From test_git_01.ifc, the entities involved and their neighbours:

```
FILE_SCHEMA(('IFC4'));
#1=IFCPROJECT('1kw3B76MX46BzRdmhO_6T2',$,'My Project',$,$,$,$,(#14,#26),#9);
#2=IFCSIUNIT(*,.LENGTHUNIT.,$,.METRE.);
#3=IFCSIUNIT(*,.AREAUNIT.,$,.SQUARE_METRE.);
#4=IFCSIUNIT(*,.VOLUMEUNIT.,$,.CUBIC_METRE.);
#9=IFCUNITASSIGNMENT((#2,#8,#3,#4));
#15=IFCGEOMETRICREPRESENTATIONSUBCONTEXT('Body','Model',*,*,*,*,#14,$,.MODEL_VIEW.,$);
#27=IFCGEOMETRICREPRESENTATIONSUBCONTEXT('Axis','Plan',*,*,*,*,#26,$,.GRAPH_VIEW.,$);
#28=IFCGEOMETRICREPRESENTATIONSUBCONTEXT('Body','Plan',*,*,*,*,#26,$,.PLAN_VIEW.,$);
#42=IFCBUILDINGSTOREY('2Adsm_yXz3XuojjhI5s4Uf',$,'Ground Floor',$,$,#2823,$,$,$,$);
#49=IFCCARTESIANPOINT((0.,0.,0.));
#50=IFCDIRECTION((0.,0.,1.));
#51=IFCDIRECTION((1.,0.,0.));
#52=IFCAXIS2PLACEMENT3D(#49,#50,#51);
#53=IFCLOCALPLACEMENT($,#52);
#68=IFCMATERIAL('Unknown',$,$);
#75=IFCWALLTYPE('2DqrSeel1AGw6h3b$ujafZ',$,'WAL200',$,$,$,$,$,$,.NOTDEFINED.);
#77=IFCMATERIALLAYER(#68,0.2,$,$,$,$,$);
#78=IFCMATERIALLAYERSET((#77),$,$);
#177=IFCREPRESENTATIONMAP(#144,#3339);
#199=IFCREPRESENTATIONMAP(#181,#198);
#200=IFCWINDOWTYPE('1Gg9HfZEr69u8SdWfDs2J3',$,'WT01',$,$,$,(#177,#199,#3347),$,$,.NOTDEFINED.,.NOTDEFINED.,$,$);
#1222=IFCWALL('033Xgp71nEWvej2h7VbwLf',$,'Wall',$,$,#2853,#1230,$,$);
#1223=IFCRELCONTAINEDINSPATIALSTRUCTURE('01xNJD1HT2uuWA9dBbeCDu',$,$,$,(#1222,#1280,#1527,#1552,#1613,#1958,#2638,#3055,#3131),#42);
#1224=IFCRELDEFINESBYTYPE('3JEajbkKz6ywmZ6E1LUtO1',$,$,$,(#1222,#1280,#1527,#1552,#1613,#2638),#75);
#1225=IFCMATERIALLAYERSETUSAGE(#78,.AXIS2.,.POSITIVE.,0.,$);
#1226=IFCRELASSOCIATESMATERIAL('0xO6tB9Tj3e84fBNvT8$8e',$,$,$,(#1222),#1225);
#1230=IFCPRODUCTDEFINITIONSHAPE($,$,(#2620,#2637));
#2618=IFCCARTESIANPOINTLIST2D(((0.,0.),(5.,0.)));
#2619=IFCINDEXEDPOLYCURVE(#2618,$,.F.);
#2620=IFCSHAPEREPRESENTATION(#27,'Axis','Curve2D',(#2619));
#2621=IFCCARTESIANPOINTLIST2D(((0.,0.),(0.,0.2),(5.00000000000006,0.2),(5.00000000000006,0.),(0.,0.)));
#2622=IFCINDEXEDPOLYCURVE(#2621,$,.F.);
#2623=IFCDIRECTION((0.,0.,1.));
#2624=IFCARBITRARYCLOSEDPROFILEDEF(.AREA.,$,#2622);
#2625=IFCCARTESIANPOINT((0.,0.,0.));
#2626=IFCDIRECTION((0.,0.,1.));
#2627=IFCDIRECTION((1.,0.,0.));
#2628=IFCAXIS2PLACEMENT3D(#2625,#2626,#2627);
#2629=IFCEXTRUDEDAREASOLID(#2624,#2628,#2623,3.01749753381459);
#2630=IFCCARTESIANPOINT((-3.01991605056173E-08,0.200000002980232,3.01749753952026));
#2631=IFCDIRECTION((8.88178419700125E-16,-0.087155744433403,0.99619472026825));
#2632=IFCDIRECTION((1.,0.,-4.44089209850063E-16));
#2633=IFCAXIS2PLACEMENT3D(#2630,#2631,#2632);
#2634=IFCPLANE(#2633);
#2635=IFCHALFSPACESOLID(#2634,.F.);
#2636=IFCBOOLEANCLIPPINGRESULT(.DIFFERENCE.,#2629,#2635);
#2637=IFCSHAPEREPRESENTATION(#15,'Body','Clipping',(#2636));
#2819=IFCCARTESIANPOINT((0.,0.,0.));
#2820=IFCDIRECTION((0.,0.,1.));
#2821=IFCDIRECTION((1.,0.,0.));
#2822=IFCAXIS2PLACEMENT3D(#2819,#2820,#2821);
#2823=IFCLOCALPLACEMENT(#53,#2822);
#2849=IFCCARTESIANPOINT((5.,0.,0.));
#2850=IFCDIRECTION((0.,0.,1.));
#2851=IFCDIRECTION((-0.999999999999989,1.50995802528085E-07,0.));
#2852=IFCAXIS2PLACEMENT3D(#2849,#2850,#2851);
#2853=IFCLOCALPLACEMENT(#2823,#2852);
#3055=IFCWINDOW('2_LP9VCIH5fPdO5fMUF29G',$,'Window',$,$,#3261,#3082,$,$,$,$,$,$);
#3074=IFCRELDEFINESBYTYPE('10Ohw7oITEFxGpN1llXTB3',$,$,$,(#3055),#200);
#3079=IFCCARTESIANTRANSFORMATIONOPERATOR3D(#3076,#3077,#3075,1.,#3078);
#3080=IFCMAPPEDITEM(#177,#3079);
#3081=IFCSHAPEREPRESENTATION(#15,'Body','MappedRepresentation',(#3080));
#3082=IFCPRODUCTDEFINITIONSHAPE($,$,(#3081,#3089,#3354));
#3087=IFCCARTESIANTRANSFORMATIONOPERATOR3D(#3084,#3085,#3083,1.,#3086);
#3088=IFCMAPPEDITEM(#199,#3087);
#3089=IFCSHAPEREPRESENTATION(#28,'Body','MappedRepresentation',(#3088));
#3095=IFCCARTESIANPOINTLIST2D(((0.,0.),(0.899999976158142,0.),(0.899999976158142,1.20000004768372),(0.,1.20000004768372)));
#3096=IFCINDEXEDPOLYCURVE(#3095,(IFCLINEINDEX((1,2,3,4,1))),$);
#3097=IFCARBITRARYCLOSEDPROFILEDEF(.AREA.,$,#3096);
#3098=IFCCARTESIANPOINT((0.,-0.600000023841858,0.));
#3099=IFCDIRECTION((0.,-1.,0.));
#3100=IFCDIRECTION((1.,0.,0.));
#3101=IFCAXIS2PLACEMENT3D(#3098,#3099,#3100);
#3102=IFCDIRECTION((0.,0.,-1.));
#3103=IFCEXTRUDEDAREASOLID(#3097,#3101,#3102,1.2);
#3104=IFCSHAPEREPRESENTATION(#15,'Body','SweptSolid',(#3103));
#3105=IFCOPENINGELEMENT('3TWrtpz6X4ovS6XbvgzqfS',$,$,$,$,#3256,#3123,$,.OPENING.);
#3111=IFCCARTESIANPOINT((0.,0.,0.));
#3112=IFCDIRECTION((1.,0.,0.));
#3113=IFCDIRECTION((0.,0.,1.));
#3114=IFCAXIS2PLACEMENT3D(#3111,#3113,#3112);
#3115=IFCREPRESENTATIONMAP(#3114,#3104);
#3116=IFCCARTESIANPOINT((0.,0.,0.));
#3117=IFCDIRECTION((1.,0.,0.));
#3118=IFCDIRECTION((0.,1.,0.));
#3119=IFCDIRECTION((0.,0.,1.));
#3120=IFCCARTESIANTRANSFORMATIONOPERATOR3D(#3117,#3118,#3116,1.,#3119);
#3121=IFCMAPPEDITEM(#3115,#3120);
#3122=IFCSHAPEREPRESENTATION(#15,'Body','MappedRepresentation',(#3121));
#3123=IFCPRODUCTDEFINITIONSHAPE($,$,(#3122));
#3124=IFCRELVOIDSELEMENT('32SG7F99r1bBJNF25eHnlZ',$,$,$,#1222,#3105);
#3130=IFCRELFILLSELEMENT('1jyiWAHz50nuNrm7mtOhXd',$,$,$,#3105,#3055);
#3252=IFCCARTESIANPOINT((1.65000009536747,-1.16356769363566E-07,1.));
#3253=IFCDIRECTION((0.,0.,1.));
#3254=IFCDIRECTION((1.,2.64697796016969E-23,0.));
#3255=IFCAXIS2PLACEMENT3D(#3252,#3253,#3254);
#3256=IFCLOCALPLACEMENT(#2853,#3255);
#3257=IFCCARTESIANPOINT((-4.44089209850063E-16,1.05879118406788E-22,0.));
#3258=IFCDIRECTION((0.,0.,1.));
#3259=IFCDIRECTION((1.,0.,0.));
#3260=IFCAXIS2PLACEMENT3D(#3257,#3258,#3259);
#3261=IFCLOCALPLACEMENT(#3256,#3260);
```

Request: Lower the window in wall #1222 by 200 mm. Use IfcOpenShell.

```python
import numpy as np
import ifcopenshell
import ifcopenshell.api.geometry
import ifcopenshell.util.placement
import ifcopenshell.util.unit

model = ifcopenshell.open("test_git_01.ifc")
unit_scale = ifcopenshell.util.unit.calculate_unit_scale(model)

window = model.by_id(3055)
opening = window.FillsVoids[0].RelatingOpeningElement
dz = -0.2 / unit_scale

shift = np.array([0.0, 0.0, dz])
# The window is placed relative to its opening, so it follows when the opening moves.
matrix = ifcopenshell.util.placement.get_local_placement(opening.ObjectPlacement)
matrix[:3, 3] += shift
ifcopenshell.api.geometry.edit_object_placement(
    model, product=opening, matrix=matrix, is_si=False, should_transform_children=True
)

print(f"moved by {dz * unit_scale:+.3f} m")

model.write("test_git_01-out.ifc")
```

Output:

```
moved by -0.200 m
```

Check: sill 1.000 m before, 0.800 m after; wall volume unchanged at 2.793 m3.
